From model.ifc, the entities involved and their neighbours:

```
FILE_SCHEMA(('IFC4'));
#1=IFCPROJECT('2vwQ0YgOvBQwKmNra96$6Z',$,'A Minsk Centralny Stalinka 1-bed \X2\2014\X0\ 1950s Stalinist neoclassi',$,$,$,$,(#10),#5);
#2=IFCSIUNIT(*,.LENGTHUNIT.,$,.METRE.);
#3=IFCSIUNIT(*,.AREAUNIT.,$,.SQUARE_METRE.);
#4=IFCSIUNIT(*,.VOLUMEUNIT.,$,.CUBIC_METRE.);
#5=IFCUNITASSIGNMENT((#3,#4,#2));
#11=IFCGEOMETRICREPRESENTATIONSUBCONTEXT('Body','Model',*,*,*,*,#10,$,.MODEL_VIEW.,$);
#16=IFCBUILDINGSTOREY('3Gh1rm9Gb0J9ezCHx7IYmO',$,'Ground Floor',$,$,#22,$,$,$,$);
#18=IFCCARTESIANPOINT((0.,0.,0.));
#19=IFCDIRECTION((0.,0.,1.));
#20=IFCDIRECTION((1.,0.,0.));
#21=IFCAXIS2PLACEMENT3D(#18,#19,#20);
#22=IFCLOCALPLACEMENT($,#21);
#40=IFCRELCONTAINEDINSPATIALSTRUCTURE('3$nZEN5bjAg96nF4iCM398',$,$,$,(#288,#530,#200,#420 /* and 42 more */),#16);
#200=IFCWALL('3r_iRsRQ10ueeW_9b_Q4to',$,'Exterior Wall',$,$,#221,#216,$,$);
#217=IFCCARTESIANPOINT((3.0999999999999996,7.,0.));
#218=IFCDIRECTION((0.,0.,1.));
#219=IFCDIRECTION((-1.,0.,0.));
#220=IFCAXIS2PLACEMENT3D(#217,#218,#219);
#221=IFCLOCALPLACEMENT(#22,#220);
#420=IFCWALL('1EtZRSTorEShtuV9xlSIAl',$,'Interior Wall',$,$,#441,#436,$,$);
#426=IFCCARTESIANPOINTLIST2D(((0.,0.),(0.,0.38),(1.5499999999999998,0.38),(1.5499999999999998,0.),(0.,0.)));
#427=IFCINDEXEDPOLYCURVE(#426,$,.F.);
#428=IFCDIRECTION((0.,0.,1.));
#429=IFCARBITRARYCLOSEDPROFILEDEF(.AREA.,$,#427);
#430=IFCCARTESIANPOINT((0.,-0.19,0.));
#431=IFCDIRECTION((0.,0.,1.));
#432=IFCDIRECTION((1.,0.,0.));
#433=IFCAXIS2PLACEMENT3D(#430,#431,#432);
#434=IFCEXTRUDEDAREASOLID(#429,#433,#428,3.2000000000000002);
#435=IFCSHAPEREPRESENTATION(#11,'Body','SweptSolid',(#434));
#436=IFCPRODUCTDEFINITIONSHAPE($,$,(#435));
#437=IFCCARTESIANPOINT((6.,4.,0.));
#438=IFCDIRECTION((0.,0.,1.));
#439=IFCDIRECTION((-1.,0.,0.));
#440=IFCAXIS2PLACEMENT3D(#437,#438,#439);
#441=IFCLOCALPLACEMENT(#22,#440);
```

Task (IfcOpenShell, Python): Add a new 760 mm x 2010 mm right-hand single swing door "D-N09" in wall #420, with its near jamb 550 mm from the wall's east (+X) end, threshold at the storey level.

```python
import numpy as np
import ifcopenshell
import ifcopenshell.api.feature
import ifcopenshell.api.geometry
import ifcopenshell.api.root
import ifcopenshell.api.spatial
import ifcopenshell.geom
import ifcopenshell.util.element
import ifcopenshell.util.placement
import ifcopenshell.util.representation
import ifcopenshell.util.shape
import ifcopenshell.util.unit

model = ifcopenshell.open("model.ifc")
unit_scale = ifcopenshell.util.unit.calculate_unit_scale(model)
settings = ifcopenshell.geom.settings()


def volume(element):
    """Net volume in cubic metres, openings subtracted."""
    shape = ifcopenshell.geom.create_shape(settings, element)
    return ifcopenshell.util.shape.get_volume(shape.geometry)


wall = model.by_id(420)
storey = ifcopenshell.util.element.get_container(wall, ifc_class="IfcBuildingStorey")
context = ifcopenshell.util.representation.get_context(model, "Model", "Body", "MODEL_VIEW")
before = volume(wall)

width, height, from_end, sill = 0.76, 2.01, 0.55, 0.0  # metres

# The wall runs along its own X axis, and the end named is its -X end.
wall_shape = ifcopenshell.geom.create_shape(settings, wall)
x, y, z = ifcopenshell.util.shape.get_vertices(wall_shape.geometry).T
start = x.min() + from_end
face, thickness = float(y.min()), float(y.max() - y.min())
wall_matrix = ifcopenshell.util.placement.get_local_placement(wall.ObjectPlacement)
level = ifcopenshell.util.placement.get_local_placement(storey.ObjectPlacement)[2, 3]


def in_wall(x, y):
    """Placement at x, y metres in the wall's axes, at sill height."""
    matrix = wall_matrix.copy()
    matrix[:, 3] = wall_matrix @ np.array([x / unit_scale, y / unit_scale, 0.0, 1.0])
    matrix[2, 3] = level + sill / unit_scale
    return matrix


# Opening: a box that overshoots both wall faces by 50 mm.
opening = ifcopenshell.api.root.create_entity(model, ifc_class="IfcOpeningElement", predefined_type="OPENING")
box = ifcopenshell.api.geometry.add_wall_representation(
    model, context=context, length=width, height=height, thickness=thickness + 0.1
)
ifcopenshell.api.geometry.assign_representation(model, product=opening, representation=box)
ifcopenshell.api.geometry.edit_object_placement(model, product=opening, matrix=in_wall(start, face - 0.05), is_si=False)
ifcopenshell.api.feature.add_feature(model, feature=opening, element=wall)

door = ifcopenshell.api.root.create_entity(model, ifc_class="IfcDoor", name="D-N09", predefined_type="DOOR")
door.OverallWidth, door.OverallHeight = width / unit_scale, height / unit_scale
door.OperationType = "SINGLE_SWING_RIGHT"
body = ifcopenshell.api.geometry.add_door_representation(
    model,
    context=context,
    overall_width=door.OverallWidth,
    overall_height=door.OverallHeight,
    operation_type="SINGLE_SWING_RIGHT",
    lining_properties={"LiningDepth": thickness / unit_scale, "ThresholdDepth": thickness / unit_scale},
)
ifcopenshell.api.geometry.assign_representation(model, product=door, representation=body)
ifcopenshell.api.spatial.assign_container(model, products=[door], relating_structure=storey)
ifcopenshell.api.feature.add_filling(model, opening=opening, element=door)

# The lining spans the wall, so the door starts at the wall face.
ifcopenshell.api.geometry.edit_object_placement(model, product=door, matrix=in_wall(start, face), is_si=False)

after = volume(wall)

print(f"wall volume {before:.3f} -> {after:.3f} m3")

model.write("model_updated.ifc")
```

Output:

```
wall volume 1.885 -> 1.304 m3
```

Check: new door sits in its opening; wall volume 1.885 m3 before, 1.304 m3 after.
